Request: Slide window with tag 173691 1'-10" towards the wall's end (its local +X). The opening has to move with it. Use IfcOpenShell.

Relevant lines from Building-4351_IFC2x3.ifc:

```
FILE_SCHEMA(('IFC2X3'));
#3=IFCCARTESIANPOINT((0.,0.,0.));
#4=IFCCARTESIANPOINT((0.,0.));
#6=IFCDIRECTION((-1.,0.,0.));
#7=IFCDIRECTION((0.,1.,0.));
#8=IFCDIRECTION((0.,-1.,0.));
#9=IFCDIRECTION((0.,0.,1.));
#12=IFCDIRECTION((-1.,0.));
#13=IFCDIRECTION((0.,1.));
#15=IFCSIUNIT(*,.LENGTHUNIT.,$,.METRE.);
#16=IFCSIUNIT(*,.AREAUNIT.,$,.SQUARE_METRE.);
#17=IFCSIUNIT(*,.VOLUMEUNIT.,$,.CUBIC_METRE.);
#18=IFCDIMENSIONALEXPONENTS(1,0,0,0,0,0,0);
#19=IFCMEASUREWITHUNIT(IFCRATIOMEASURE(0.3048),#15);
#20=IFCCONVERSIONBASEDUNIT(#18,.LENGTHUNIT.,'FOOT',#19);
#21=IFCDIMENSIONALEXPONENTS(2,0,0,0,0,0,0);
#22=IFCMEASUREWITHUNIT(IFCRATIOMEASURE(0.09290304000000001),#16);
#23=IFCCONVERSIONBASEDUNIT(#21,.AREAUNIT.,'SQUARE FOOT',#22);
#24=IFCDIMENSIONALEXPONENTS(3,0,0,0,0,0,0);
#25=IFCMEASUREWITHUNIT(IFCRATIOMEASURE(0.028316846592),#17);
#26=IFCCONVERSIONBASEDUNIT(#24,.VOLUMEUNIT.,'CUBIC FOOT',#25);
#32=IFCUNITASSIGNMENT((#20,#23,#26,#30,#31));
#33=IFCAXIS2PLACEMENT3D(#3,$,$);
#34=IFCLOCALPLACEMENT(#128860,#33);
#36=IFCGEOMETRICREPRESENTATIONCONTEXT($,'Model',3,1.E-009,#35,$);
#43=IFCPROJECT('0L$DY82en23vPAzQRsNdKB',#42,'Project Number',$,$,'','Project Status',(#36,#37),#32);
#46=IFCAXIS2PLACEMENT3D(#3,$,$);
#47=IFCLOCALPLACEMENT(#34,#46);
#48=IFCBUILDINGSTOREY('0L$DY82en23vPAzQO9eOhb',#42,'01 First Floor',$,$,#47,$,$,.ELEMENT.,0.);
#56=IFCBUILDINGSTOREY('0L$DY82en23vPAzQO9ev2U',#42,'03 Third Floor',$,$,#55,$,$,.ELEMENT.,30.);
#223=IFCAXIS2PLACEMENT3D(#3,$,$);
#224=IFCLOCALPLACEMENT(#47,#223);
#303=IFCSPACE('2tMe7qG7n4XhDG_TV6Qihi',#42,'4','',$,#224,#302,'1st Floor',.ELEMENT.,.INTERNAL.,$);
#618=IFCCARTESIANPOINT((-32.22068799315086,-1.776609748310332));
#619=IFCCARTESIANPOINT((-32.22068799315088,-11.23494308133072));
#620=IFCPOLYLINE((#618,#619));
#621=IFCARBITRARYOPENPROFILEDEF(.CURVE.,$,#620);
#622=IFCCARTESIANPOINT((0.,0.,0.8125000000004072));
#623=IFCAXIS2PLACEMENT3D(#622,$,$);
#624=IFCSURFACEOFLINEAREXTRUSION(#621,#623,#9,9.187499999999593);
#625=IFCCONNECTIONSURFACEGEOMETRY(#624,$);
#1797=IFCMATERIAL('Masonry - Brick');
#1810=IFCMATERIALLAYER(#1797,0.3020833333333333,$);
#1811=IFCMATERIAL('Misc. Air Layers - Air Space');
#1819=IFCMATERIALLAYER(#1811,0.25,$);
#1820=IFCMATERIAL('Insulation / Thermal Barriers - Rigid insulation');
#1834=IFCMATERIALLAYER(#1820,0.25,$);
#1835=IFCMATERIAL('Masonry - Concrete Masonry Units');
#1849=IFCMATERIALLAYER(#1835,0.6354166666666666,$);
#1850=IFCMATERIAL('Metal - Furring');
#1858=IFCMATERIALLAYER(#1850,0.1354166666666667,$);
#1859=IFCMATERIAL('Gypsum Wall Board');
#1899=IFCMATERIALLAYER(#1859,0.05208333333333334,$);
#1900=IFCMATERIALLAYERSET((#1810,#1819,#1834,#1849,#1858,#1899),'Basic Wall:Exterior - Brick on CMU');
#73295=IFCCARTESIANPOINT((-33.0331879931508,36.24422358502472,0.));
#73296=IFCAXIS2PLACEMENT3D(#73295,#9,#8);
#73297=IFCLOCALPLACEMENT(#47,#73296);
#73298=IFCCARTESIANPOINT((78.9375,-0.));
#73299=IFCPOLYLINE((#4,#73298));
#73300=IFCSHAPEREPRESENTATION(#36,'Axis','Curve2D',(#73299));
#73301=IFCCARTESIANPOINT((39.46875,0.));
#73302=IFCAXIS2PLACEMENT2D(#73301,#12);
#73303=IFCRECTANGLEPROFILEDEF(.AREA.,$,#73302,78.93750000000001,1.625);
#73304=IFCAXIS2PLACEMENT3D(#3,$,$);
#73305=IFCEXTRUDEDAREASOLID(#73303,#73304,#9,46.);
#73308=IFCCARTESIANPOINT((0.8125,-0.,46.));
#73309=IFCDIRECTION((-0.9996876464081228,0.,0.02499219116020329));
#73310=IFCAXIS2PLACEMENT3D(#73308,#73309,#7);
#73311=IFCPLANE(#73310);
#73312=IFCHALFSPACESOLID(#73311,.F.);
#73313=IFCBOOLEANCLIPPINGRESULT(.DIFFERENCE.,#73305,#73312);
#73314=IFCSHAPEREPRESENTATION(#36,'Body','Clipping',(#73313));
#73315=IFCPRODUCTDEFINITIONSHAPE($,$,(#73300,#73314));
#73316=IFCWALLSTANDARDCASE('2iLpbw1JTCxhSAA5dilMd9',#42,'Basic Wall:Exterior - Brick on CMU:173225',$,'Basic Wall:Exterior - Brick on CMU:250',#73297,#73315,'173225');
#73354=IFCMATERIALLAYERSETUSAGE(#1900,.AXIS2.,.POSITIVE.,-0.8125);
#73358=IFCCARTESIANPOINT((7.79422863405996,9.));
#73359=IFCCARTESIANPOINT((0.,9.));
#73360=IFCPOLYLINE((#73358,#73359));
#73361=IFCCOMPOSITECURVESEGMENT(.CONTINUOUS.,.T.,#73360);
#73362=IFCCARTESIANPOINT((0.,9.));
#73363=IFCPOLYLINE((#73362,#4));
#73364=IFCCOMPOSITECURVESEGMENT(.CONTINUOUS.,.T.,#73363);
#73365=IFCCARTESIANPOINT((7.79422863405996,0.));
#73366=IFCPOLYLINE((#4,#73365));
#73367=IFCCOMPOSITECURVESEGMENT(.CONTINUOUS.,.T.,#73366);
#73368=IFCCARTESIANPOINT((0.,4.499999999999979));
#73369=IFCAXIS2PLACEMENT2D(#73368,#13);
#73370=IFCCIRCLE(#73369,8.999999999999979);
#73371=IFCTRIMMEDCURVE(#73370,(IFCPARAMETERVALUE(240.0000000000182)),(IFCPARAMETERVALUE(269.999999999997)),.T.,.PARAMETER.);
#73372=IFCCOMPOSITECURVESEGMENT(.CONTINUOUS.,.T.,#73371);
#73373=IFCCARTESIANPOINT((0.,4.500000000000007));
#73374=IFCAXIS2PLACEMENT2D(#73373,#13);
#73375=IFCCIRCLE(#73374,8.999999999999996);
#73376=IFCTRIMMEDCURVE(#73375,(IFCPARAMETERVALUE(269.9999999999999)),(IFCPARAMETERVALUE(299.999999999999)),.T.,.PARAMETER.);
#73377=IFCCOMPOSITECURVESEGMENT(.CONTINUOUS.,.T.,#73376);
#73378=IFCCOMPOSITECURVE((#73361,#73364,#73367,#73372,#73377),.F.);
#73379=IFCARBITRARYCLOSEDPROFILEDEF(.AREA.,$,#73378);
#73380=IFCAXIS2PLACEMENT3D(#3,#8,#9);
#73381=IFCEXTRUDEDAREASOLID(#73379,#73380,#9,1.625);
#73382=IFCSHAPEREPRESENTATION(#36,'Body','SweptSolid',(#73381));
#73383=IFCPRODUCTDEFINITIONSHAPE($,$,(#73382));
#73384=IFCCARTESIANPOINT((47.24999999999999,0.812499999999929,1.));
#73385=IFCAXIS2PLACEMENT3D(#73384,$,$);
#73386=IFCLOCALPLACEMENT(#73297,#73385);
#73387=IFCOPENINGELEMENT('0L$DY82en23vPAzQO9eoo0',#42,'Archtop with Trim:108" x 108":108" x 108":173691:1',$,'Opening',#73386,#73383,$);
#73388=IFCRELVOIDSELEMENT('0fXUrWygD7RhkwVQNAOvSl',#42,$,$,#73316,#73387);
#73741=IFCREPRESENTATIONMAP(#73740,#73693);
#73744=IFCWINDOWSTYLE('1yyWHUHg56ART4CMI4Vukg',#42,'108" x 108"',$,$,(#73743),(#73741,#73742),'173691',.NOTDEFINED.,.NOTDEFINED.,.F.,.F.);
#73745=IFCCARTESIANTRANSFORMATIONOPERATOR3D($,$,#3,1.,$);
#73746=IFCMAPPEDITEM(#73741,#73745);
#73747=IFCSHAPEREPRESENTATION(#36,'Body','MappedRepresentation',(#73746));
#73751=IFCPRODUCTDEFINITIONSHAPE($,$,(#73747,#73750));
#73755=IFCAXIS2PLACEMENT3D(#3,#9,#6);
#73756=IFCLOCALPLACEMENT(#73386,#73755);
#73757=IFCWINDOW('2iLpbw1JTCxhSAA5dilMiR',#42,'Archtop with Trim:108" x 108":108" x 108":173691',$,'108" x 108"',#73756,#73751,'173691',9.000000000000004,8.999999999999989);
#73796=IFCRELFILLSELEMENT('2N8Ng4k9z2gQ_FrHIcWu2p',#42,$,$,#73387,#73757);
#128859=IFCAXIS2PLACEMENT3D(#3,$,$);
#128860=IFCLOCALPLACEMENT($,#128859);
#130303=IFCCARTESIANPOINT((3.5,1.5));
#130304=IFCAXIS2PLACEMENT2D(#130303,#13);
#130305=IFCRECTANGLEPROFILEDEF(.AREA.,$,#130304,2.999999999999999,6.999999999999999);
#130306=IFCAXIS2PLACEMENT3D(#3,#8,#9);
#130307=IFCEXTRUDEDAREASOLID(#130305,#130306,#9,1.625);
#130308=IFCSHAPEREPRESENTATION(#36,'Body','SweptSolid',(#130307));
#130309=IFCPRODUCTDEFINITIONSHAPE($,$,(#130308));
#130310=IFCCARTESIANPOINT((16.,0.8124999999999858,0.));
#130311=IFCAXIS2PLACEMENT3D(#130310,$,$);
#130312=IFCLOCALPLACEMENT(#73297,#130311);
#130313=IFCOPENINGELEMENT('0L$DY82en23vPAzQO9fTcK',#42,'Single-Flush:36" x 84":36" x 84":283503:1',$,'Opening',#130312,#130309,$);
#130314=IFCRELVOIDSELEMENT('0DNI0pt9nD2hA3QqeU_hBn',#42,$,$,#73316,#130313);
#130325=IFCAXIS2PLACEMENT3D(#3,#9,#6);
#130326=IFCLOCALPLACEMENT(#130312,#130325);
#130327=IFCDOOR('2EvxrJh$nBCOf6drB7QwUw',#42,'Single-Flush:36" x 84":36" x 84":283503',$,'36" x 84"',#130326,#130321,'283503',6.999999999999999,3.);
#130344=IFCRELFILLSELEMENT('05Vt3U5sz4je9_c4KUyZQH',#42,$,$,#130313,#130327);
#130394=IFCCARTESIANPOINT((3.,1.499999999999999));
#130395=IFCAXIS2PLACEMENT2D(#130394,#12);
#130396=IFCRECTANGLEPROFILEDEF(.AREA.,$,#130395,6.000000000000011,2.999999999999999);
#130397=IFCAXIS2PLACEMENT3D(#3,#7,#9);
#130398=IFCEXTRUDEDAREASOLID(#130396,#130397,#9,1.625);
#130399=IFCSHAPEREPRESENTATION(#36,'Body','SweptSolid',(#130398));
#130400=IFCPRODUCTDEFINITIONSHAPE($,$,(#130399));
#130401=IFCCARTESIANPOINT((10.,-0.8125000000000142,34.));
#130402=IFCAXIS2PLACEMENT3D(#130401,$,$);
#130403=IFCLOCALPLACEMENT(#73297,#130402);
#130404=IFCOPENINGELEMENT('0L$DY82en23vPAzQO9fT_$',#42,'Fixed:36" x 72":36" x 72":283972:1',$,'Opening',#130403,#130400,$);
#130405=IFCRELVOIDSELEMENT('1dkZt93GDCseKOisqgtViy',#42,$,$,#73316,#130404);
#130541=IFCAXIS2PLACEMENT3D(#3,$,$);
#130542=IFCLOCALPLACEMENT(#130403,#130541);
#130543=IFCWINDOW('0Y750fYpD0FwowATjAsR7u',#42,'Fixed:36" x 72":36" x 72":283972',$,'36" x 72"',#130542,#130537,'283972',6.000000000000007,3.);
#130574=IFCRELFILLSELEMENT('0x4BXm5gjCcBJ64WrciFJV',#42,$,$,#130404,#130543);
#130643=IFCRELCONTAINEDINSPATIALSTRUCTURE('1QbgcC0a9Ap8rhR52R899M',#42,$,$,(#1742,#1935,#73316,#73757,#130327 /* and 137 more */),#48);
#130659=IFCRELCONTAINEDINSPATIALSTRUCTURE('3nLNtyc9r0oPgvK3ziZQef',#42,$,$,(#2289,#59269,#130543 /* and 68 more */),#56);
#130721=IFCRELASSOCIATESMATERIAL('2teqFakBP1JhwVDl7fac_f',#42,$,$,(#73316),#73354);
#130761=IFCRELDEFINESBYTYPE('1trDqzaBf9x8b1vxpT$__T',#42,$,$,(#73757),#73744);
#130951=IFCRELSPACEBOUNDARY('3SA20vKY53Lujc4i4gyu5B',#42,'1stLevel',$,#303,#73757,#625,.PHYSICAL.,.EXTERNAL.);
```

```python
import numpy as np
import ifcopenshell
import ifcopenshell.api.geometry
import ifcopenshell.util.placement
import ifcopenshell.util.unit

model = ifcopenshell.open("Building-4351_IFC2x3.ifc")
unit_scale = ifcopenshell.util.unit.calculate_unit_scale(model)

window = model.by_guid("2iLpbw1JTCxhSAA5dilMiR")
opening = window.FillsVoids[0].RelatingOpeningElement
wall = opening.VoidsElements[0].RelatingBuildingElement

wall_matrix = ifcopenshell.util.placement.get_local_placement(wall.ObjectPlacement)
shift = wall_matrix[:3, 0] * 22 * 0.0254 / unit_scale
before = ifcopenshell.util.placement.get_local_placement(window.ObjectPlacement)[:3, 3].copy()

# The window is placed relative to its opening, so it follows when the opening moves.
matrix = ifcopenshell.util.placement.get_local_placement(opening.ObjectPlacement)
matrix[:3, 3] += shift
ifcopenshell.api.geometry.edit_object_placement(
    model, product=opening, matrix=matrix, is_si=False, should_transform_children=True
)

# Space boundary surfaces are stored in each space's coordinates; move them too.
for rel in window.ProvidesBoundaries:
    if not rel.ConnectionGeometry:
        continue
    surface = rel.ConnectionGeometry.SurfaceOnRelatingElement
    space_matrix = ifcopenshell.util.placement.get_local_placement(rel.RelatingSpace.ObjectPlacement)
    point = np.array(surface.Position.Location.Coordinates) + space_matrix[:3, :3].T @ shift
    surface.Position = model.createIfcAxis2Placement3D(
        model.createIfcCartesianPoint(point.tolist()), surface.Position.Axis, surface.Position.RefDirection
    )

after = ifcopenshell.util.placement.get_local_placement(window.ObjectPlacement)[:3, 3]
print("window moved by", (after - before).round(3) + 0.0)

model.write("Building-4351_IFC2x3_updated.ifc")
```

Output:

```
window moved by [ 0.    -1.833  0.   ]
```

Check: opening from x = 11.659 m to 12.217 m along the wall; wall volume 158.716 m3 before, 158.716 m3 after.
